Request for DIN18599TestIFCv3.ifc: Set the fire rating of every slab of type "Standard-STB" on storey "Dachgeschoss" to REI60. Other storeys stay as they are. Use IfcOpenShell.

First a look at what the model holds.

```python
import ifcopenshell
import ifcopenshell.util.element

model = ifcopenshell.open("DIN18599TestIFCv3.ifc")
print(model.schema)
storey = next(s for s in model.by_type("IfcBuildingStorey") if s.Name == "Dachgeschoss")
slabs = [e for e in ifcopenshell.util.element.get_decomposition(storey) if e.is_a("IfcSlab")]
seen = {}
for e in slabs:
    element_type = ifcopenshell.util.element.get_type(e)
    key = (element_type.Name if element_type != e and element_type else None, ifcopenshell.util.element.get_pset(e, "Pset_SlabCommon", "FireRating"))
    seen[key] = seen.get(key, 0) + 1
for (name, value), count in sorted(seen.items(), key=str):
    print(count, "x", name, "|", value)
```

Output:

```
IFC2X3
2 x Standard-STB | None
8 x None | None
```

```python
import ifcopenshell
import ifcopenshell.api.pset
import ifcopenshell.util.element

model = ifcopenshell.open("DIN18599TestIFCv3.ifc")

storey = next(s for s in model.by_type("IfcBuildingStorey") if s.Name == "Dachgeschoss")
slabs = [e for e in ifcopenshell.util.element.get_decomposition(storey) if e.is_a("IfcSlab")]

count = 0
for e in slabs:
    element_type = ifcopenshell.util.element.get_type(e)
    if element_type in (None, e) or element_type.Name != "Standard-STB":
        continue
    # add_pset returns the element's existing set when there is one.
    pset = ifcopenshell.api.pset.add_pset(model, product=e, name="Pset_SlabCommon")
    ifcopenshell.api.pset.edit_pset(model, pset=pset, properties={"FireRating": "REI60"})
    count += 1

print(count, "slabs updated")

model.write("DIN18599TestIFCv3_rev.ifc")
```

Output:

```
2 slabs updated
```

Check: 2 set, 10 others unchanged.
